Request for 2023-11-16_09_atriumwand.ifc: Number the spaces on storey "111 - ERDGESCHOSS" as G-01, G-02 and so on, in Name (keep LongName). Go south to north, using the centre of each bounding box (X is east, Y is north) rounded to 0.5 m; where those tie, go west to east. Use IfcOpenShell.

First a look at what the model holds.

```python
import ifcopenshell
import ifcopenshell.util.element
import ifcopenshell.util.placement

model = ifcopenshell.open("2023-11-16_09_atriumwand.ifc")
print(model.schema)
storey = next(s for s in model.by_type("IfcBuildingStorey") if s.Name == "111 - ERDGESCHOSS")
spaces = [e for e in ifcopenshell.util.element.get_decomposition(storey) if e.is_a("IfcSpace")]
for e in sorted(spaces, key=lambda e: e.id()):
    origin = ifcopenshell.util.placement.get_local_placement(e.ObjectPlacement)[:3, 3]
    print(e.id(), e.Name, e.LongName, origin.round(2) + 0.0, sep=" | ")
```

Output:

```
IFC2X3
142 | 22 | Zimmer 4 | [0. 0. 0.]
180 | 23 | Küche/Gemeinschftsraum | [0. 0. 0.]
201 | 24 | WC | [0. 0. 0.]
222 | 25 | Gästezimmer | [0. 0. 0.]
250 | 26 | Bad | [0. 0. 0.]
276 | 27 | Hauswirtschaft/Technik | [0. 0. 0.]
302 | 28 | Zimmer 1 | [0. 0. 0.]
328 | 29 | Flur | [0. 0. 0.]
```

```python
import ifcopenshell
import ifcopenshell.geom
import ifcopenshell.util.element
import ifcopenshell.util.shape

model = ifcopenshell.open("2023-11-16_09_atriumwand.ifc")
settings = ifcopenshell.geom.settings()
settings.set("use-world-coords", True)


def centre(element):
    shape = ifcopenshell.geom.create_shape(settings, element)
    return ifcopenshell.util.shape.get_bbox_centroid(shape.geometry)


storey = next(s for s in model.by_type("IfcBuildingStorey") if s.Name == "111 - ERDGESCHOSS")
spaces = [e for e in ifcopenshell.util.element.get_decomposition(storey) if e.is_a("IfcSpace")]

# Insertion points can sit at a corner or the storey origin, so sort by the geometry (in metres).
centres = {e: centre(e) for e in spaces}
spaces.sort(key=lambda e: (round(centres[e][1] / 0.5), centres[e][0]))

for i, e in enumerate(spaces, start=1):
    number = f"G-{i:02d}"
    e.Name = number
    print(e.id(), number)

model.write("2023-11-16_09_atriumwand-out.ifc")
```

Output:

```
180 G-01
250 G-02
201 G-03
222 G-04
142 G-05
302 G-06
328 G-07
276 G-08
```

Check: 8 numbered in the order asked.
